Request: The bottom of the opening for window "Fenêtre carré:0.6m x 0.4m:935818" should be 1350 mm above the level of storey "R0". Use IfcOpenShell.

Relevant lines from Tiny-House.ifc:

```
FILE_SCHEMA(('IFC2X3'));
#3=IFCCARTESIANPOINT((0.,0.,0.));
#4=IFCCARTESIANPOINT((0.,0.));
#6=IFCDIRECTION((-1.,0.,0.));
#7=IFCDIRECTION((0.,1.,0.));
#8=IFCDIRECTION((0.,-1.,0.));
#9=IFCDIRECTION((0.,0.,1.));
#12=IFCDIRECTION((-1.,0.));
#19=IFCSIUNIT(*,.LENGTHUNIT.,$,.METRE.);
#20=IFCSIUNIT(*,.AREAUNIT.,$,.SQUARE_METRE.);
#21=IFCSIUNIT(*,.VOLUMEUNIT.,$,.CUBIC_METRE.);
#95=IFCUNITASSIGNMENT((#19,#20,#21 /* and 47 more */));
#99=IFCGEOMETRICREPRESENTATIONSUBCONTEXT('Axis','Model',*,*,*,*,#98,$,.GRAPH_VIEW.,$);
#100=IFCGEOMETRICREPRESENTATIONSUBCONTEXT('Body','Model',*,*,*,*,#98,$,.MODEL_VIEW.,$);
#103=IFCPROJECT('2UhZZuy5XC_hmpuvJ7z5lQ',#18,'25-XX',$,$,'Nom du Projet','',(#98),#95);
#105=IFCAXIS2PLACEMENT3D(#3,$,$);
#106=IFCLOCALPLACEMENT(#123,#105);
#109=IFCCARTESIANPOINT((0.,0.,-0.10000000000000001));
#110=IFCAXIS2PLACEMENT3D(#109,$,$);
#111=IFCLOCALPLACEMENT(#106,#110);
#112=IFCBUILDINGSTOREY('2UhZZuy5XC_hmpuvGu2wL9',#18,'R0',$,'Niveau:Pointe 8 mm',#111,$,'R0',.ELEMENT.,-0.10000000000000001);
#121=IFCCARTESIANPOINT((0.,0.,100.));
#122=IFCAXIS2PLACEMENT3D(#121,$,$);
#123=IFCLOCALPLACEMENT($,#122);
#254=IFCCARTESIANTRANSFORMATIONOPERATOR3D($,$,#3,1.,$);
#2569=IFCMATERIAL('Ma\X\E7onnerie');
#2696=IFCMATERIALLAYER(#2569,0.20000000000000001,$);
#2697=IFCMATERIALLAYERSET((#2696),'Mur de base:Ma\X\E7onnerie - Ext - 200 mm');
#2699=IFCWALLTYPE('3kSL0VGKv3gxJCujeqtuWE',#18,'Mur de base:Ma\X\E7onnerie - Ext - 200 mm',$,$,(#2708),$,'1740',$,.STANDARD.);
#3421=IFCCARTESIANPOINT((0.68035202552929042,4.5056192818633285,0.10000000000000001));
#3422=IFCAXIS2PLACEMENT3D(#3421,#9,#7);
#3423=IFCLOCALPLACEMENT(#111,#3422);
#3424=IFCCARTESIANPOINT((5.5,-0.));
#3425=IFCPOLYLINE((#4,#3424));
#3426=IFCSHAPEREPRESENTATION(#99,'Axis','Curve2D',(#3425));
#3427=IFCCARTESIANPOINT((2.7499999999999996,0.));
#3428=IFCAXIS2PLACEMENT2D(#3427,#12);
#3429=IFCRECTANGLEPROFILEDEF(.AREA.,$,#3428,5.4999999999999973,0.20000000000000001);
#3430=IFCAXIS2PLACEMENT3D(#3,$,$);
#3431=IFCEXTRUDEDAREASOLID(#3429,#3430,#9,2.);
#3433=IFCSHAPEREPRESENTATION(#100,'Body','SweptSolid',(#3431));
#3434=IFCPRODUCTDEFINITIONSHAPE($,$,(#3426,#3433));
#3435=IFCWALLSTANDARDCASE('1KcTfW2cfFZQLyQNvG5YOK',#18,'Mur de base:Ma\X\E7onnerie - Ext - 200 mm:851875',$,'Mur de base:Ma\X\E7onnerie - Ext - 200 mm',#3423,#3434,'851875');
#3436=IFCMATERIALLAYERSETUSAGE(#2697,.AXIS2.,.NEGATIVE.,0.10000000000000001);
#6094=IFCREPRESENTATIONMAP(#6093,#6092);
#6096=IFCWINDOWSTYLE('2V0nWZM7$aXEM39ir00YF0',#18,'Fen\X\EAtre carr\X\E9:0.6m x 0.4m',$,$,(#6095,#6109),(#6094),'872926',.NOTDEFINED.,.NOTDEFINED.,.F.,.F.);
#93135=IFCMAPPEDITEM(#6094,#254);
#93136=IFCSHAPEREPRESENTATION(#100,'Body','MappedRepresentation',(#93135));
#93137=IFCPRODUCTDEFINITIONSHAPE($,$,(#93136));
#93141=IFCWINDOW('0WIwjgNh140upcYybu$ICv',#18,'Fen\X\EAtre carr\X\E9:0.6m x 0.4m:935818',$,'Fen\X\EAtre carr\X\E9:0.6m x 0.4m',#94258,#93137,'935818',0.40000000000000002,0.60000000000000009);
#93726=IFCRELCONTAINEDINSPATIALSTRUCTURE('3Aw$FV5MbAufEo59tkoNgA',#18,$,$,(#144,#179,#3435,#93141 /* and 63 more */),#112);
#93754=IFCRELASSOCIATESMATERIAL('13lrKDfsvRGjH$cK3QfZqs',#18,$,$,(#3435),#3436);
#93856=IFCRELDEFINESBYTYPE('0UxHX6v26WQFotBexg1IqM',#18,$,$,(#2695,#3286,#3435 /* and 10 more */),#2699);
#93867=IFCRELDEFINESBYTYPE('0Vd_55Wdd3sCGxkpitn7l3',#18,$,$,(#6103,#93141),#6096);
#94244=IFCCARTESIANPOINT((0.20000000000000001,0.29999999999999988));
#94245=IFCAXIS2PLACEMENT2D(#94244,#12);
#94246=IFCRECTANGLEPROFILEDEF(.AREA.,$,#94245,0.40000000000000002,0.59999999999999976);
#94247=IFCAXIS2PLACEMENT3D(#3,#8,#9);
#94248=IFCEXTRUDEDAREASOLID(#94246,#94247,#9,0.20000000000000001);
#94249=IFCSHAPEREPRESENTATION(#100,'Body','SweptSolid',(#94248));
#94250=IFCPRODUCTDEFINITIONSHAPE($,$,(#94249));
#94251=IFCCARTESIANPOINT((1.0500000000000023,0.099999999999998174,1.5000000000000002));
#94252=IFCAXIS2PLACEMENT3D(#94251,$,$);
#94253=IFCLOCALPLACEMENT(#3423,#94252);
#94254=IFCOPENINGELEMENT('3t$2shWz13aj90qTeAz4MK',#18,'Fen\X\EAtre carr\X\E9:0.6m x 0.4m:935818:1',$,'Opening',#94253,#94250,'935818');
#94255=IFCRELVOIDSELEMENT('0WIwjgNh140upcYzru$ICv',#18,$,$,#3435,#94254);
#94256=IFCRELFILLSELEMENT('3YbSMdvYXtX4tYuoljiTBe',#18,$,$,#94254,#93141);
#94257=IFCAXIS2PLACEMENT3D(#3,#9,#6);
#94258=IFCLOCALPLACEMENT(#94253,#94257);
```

```python
import numpy as np
import ifcopenshell
import ifcopenshell.api.geometry
import ifcopenshell.geom
import ifcopenshell.util.element
import ifcopenshell.util.placement
import ifcopenshell.util.shape
import ifcopenshell.util.unit

model = ifcopenshell.open("Tiny-House.ifc")
unit_scale = ifcopenshell.util.unit.calculate_unit_scale(model)

window = model.by_guid("0WIwjgNh140upcYybu$ICv")
opening = window.FillsVoids[0].RelatingOpeningElement
storey = ifcopenshell.util.element.get_container(window, ifc_class="IfcBuildingStorey")
level = ifcopenshell.util.placement.get_local_placement(storey.ObjectPlacement)[2, 3]

# The opening's origin need not be at the sill, so measure its lowest point.
shape = ifcopenshell.geom.create_shape(ifcopenshell.geom.settings(), opening)
bottom = ifcopenshell.util.shape.get_shape_bottom_elevation(shape, shape.geometry) / unit_scale
dz = level + 1.35 / unit_scale - bottom

shift = np.array([0.0, 0.0, dz])
# The window is placed relative to its opening, so it follows when the opening moves.
matrix = ifcopenshell.util.placement.get_local_placement(opening.ObjectPlacement)
matrix[:3, 3] += shift
ifcopenshell.api.geometry.edit_object_placement(
    model, product=opening, matrix=matrix, is_si=False, should_transform_children=True
)

print(f"moved by {dz * unit_scale:+.3f} m")

model.write("Tiny-House-out.ifc")
```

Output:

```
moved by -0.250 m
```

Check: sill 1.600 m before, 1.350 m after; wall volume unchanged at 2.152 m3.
